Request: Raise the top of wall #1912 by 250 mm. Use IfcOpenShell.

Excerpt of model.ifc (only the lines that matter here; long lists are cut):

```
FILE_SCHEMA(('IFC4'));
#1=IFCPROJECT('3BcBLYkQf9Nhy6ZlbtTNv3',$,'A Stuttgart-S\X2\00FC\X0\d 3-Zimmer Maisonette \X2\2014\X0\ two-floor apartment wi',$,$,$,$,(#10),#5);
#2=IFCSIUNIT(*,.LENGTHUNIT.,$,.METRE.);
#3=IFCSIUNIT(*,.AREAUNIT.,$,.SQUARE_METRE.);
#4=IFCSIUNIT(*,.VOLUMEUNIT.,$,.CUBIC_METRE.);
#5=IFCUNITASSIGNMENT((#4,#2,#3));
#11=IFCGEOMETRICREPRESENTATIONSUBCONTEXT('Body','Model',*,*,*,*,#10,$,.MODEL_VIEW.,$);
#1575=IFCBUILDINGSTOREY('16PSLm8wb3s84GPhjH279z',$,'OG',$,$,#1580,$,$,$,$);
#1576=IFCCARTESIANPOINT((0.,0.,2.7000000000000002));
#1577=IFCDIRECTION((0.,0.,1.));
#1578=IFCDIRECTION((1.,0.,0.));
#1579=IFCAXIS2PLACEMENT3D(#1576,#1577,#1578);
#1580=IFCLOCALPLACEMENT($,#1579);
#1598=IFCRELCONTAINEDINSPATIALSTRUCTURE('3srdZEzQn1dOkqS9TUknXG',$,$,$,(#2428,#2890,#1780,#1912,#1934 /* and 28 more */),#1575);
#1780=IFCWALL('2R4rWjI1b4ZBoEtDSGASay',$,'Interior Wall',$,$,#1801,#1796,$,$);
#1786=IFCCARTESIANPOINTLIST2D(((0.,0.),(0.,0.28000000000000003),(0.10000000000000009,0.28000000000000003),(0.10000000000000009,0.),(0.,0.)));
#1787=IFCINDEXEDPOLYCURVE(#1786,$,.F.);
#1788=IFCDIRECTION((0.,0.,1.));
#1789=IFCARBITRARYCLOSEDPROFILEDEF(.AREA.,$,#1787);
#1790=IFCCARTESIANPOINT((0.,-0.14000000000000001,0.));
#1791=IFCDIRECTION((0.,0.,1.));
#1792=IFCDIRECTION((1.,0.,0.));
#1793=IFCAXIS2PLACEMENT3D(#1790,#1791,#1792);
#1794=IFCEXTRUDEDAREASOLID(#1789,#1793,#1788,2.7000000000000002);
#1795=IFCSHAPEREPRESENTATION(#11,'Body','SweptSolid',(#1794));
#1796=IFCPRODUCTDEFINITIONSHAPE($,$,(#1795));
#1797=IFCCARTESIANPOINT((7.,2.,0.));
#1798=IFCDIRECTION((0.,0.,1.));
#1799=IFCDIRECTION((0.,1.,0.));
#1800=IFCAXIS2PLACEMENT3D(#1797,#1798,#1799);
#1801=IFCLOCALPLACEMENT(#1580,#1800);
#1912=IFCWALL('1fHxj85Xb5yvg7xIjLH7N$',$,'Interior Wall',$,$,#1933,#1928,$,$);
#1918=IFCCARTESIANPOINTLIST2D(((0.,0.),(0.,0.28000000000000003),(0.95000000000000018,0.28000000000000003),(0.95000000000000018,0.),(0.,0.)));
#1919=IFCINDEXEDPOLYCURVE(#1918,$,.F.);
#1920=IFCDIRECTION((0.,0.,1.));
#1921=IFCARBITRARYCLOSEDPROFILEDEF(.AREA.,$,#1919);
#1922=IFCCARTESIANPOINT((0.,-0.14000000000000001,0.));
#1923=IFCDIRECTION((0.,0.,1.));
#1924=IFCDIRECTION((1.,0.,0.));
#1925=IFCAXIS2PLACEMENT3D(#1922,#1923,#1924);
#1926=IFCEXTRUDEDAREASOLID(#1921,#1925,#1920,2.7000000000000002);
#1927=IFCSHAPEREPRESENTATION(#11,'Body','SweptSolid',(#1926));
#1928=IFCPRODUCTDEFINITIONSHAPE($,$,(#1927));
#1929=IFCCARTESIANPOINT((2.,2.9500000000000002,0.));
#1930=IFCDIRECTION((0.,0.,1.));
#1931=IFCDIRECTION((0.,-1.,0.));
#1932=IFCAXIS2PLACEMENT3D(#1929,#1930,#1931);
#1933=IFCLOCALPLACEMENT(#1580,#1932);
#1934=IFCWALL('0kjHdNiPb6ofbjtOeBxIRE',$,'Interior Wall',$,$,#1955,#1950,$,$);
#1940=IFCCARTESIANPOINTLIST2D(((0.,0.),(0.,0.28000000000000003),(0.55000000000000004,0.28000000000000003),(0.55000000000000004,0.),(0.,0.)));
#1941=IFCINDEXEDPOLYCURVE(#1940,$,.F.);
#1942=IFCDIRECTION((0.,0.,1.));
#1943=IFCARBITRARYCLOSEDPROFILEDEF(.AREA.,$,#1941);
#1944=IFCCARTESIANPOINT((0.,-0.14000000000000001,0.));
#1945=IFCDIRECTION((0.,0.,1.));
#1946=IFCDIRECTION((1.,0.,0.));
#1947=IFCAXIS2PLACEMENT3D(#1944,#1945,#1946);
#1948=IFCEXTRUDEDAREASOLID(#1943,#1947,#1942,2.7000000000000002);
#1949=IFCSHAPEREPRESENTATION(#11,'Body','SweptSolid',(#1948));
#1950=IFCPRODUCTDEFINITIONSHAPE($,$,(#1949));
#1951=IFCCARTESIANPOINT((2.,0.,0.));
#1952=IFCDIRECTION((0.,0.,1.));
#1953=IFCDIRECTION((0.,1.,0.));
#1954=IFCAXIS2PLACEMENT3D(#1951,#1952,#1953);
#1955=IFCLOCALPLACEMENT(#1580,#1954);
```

```python
import ifcopenshell
import ifcopenshell.geom
import ifcopenshell.util.representation
import ifcopenshell.util.shape
import ifcopenshell.util.unit

model = ifcopenshell.open("model.ifc")
unit_scale = ifcopenshell.util.unit.calculate_unit_scale(model)
settings = ifcopenshell.geom.settings()


def volume(element):
    """Net volume in cubic metres, openings subtracted."""
    shape = ifcopenshell.geom.create_shape(settings, element)
    return ifcopenshell.util.shape.get_volume(shape.geometry)


wall = model.by_guid("1fHxj85Xb5yvg7xIjLH7N$")
before = volume(wall)

body = ifcopenshell.util.representation.get_representation(wall, "Model", "Body")
solid = body.Items[0]
old_height = solid.Depth
solid.Depth += 0.25 / unit_scale
after = volume(wall)

print(f"height {old_height:g} -> {solid.Depth:g}, volume {before:.3f} -> {after:.3f} m3")

model.write("model_updated.ifc")
```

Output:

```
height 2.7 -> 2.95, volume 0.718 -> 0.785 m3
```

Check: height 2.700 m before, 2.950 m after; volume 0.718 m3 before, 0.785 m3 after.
